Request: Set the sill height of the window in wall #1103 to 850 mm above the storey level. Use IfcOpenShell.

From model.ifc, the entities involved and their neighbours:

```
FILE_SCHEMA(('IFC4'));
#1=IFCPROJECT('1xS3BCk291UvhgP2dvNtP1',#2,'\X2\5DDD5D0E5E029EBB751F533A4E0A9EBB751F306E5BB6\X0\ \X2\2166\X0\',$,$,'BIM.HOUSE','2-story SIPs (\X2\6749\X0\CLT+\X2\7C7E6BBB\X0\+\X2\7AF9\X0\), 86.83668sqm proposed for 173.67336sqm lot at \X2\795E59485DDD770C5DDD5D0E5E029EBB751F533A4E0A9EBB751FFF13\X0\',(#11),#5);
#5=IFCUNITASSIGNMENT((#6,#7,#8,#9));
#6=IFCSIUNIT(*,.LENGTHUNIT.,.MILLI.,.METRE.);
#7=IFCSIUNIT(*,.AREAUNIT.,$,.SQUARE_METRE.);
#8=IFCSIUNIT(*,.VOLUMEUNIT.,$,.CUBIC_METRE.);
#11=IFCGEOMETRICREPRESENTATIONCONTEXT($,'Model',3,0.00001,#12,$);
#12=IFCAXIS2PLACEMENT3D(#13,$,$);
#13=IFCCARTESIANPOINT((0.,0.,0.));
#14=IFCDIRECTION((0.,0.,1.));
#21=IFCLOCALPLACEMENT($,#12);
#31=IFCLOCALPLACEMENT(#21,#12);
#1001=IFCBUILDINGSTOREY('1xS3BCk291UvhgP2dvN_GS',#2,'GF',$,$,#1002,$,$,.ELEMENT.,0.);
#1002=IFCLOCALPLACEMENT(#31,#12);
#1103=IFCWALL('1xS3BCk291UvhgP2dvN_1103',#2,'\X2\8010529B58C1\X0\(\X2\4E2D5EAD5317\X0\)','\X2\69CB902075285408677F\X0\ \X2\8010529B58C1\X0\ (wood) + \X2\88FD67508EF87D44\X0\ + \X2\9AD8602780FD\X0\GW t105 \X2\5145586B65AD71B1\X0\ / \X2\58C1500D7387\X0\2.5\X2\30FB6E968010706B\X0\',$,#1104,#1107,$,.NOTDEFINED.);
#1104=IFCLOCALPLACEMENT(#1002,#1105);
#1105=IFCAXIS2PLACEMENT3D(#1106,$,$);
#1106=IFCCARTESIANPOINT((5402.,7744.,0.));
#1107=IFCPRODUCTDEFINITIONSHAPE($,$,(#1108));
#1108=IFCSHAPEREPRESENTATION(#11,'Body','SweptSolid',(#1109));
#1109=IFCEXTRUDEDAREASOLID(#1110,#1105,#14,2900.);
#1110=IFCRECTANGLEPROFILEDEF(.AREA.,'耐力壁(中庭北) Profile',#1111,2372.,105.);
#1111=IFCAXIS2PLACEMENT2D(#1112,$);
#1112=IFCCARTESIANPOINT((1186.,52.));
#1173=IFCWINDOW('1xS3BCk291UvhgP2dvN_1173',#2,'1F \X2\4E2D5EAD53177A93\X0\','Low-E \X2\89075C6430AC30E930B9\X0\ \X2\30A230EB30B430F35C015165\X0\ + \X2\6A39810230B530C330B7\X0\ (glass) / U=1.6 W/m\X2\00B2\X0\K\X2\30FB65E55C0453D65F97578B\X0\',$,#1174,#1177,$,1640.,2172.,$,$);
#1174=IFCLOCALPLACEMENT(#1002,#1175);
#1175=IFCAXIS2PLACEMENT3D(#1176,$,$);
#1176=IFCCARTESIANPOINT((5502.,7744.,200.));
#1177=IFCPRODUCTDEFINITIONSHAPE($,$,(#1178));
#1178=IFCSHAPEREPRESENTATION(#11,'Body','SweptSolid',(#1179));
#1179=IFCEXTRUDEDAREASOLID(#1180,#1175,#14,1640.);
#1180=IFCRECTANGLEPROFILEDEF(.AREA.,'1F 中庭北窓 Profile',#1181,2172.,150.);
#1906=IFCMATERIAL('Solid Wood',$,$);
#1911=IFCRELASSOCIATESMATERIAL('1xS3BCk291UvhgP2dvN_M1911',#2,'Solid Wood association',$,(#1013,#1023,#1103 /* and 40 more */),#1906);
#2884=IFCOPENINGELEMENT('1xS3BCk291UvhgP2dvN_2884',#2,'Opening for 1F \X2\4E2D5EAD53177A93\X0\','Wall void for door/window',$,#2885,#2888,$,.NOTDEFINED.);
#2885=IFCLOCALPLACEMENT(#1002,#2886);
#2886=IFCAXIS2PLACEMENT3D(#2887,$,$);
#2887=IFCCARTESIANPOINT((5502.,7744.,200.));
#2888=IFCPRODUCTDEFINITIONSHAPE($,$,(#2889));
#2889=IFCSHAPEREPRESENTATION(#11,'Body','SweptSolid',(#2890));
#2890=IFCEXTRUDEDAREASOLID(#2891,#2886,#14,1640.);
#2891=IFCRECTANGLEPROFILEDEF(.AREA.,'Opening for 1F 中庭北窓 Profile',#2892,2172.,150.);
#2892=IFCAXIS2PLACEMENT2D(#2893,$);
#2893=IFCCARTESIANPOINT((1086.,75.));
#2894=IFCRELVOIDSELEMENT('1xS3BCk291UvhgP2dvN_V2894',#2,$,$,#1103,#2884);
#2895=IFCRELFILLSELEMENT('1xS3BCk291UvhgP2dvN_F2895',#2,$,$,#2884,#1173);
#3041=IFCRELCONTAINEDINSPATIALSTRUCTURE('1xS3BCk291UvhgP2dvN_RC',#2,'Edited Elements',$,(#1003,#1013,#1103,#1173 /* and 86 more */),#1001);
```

```python
import numpy as np
import ifcopenshell
import ifcopenshell.api.geometry
import ifcopenshell.geom
import ifcopenshell.util.element
import ifcopenshell.util.placement
import ifcopenshell.util.shape
import ifcopenshell.util.unit

model = ifcopenshell.open("model.ifc")
unit_scale = ifcopenshell.util.unit.calculate_unit_scale(model)

window = model.by_guid("1xS3BCk291UvhgP2dvN_1173")
opening = window.FillsVoids[0].RelatingOpeningElement
storey = ifcopenshell.util.element.get_container(window, ifc_class="IfcBuildingStorey")
level = ifcopenshell.util.placement.get_local_placement(storey.ObjectPlacement)[2, 3]

# The opening's origin need not be at the sill, so measure its lowest point.
shape = ifcopenshell.geom.create_shape(ifcopenshell.geom.settings(), opening)
bottom = ifcopenshell.util.shape.get_shape_bottom_elevation(shape, shape.geometry) / unit_scale
dz = level + 0.85 / unit_scale - bottom

shift = np.array([0.0, 0.0, dz])
# The window is not placed relative to its opening, so move both.
for product in (opening, window):
    matrix = ifcopenshell.util.placement.get_local_placement(product.ObjectPlacement)
    matrix[:3, 3] += shift
    ifcopenshell.api.geometry.edit_object_placement(model, product=product, matrix=matrix, is_si=False)

print(f"moved by {dz * unit_scale:+.3f} m")

model.write("model_v2.ifc")
```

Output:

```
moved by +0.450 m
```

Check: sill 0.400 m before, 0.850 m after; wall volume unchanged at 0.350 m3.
